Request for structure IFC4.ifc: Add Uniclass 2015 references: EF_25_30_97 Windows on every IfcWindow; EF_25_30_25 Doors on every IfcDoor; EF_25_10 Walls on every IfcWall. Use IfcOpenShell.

First a look at what the model holds.

```python
import ifcopenshell

model = ifcopenshell.open("structure IFC4.ifc")
print(model.schema)
print("classifications:", [c.Name for c in model.by_type("IfcClassification")])
for ifc_class in ("IfcDoor", "IfcRoof", "IfcStair", "IfcWall", "IfcWindow"):
    print(ifc_class, len(model.by_type(ifc_class)))
```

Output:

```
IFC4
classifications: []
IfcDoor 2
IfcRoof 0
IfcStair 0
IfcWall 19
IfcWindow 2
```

```python
import ifcopenshell
import ifcopenshell.api.classification

model = ifcopenshell.open("structure IFC4.ifc")

system = ifcopenshell.api.classification.add_classification(model, classification="Uniclass 2015")

codes = {
    "IfcWindow": ("EF_25_30_97", "Windows"),
    "IfcDoor": ("EF_25_30_25", "Doors"),
    "IfcWall": ("EF_25_10", "Walls"),
}
for ifc_class, (code, name) in codes.items():
    products = model.by_type(ifc_class)
    ifcopenshell.api.classification.add_reference(
        model, products=products, classification=system, identification=code, name=name
    )
    print(code, len(products))

model.write("structure IFC4_edited.ifc")
```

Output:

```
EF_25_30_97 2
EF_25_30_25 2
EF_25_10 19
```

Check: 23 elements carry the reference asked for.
